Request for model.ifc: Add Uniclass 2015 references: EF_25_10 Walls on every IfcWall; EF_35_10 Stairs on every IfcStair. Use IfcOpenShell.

First a look at what the model holds.

```python
import ifcopenshell

model = ifcopenshell.open("model.ifc")
print(model.schema)
print("classifications:", [c.Name for c in model.by_type("IfcClassification")])
for ifc_class in ("IfcDoor", "IfcRoof", "IfcStair", "IfcWall", "IfcWindow"):
    print(ifc_class, len(model.by_type(ifc_class)))
```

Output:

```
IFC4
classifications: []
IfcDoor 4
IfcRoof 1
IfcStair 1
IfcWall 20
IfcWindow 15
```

```python
import ifcopenshell
import ifcopenshell.api.classification

model = ifcopenshell.open("model.ifc")

system = ifcopenshell.api.classification.add_classification(model, classification="Uniclass 2015")

codes = {
    "IfcWall": ("EF_25_10", "Walls"),
    "IfcStair": ("EF_35_10", "Stairs"),
}
for ifc_class, (code, name) in codes.items():
    products = model.by_type(ifc_class)
    ifcopenshell.api.classification.add_reference(
        model, products=products, classification=system, identification=code, name=name
    )
    print(code, len(products))

model.write("model_v2.ifc")
```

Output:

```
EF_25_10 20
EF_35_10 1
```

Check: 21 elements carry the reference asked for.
